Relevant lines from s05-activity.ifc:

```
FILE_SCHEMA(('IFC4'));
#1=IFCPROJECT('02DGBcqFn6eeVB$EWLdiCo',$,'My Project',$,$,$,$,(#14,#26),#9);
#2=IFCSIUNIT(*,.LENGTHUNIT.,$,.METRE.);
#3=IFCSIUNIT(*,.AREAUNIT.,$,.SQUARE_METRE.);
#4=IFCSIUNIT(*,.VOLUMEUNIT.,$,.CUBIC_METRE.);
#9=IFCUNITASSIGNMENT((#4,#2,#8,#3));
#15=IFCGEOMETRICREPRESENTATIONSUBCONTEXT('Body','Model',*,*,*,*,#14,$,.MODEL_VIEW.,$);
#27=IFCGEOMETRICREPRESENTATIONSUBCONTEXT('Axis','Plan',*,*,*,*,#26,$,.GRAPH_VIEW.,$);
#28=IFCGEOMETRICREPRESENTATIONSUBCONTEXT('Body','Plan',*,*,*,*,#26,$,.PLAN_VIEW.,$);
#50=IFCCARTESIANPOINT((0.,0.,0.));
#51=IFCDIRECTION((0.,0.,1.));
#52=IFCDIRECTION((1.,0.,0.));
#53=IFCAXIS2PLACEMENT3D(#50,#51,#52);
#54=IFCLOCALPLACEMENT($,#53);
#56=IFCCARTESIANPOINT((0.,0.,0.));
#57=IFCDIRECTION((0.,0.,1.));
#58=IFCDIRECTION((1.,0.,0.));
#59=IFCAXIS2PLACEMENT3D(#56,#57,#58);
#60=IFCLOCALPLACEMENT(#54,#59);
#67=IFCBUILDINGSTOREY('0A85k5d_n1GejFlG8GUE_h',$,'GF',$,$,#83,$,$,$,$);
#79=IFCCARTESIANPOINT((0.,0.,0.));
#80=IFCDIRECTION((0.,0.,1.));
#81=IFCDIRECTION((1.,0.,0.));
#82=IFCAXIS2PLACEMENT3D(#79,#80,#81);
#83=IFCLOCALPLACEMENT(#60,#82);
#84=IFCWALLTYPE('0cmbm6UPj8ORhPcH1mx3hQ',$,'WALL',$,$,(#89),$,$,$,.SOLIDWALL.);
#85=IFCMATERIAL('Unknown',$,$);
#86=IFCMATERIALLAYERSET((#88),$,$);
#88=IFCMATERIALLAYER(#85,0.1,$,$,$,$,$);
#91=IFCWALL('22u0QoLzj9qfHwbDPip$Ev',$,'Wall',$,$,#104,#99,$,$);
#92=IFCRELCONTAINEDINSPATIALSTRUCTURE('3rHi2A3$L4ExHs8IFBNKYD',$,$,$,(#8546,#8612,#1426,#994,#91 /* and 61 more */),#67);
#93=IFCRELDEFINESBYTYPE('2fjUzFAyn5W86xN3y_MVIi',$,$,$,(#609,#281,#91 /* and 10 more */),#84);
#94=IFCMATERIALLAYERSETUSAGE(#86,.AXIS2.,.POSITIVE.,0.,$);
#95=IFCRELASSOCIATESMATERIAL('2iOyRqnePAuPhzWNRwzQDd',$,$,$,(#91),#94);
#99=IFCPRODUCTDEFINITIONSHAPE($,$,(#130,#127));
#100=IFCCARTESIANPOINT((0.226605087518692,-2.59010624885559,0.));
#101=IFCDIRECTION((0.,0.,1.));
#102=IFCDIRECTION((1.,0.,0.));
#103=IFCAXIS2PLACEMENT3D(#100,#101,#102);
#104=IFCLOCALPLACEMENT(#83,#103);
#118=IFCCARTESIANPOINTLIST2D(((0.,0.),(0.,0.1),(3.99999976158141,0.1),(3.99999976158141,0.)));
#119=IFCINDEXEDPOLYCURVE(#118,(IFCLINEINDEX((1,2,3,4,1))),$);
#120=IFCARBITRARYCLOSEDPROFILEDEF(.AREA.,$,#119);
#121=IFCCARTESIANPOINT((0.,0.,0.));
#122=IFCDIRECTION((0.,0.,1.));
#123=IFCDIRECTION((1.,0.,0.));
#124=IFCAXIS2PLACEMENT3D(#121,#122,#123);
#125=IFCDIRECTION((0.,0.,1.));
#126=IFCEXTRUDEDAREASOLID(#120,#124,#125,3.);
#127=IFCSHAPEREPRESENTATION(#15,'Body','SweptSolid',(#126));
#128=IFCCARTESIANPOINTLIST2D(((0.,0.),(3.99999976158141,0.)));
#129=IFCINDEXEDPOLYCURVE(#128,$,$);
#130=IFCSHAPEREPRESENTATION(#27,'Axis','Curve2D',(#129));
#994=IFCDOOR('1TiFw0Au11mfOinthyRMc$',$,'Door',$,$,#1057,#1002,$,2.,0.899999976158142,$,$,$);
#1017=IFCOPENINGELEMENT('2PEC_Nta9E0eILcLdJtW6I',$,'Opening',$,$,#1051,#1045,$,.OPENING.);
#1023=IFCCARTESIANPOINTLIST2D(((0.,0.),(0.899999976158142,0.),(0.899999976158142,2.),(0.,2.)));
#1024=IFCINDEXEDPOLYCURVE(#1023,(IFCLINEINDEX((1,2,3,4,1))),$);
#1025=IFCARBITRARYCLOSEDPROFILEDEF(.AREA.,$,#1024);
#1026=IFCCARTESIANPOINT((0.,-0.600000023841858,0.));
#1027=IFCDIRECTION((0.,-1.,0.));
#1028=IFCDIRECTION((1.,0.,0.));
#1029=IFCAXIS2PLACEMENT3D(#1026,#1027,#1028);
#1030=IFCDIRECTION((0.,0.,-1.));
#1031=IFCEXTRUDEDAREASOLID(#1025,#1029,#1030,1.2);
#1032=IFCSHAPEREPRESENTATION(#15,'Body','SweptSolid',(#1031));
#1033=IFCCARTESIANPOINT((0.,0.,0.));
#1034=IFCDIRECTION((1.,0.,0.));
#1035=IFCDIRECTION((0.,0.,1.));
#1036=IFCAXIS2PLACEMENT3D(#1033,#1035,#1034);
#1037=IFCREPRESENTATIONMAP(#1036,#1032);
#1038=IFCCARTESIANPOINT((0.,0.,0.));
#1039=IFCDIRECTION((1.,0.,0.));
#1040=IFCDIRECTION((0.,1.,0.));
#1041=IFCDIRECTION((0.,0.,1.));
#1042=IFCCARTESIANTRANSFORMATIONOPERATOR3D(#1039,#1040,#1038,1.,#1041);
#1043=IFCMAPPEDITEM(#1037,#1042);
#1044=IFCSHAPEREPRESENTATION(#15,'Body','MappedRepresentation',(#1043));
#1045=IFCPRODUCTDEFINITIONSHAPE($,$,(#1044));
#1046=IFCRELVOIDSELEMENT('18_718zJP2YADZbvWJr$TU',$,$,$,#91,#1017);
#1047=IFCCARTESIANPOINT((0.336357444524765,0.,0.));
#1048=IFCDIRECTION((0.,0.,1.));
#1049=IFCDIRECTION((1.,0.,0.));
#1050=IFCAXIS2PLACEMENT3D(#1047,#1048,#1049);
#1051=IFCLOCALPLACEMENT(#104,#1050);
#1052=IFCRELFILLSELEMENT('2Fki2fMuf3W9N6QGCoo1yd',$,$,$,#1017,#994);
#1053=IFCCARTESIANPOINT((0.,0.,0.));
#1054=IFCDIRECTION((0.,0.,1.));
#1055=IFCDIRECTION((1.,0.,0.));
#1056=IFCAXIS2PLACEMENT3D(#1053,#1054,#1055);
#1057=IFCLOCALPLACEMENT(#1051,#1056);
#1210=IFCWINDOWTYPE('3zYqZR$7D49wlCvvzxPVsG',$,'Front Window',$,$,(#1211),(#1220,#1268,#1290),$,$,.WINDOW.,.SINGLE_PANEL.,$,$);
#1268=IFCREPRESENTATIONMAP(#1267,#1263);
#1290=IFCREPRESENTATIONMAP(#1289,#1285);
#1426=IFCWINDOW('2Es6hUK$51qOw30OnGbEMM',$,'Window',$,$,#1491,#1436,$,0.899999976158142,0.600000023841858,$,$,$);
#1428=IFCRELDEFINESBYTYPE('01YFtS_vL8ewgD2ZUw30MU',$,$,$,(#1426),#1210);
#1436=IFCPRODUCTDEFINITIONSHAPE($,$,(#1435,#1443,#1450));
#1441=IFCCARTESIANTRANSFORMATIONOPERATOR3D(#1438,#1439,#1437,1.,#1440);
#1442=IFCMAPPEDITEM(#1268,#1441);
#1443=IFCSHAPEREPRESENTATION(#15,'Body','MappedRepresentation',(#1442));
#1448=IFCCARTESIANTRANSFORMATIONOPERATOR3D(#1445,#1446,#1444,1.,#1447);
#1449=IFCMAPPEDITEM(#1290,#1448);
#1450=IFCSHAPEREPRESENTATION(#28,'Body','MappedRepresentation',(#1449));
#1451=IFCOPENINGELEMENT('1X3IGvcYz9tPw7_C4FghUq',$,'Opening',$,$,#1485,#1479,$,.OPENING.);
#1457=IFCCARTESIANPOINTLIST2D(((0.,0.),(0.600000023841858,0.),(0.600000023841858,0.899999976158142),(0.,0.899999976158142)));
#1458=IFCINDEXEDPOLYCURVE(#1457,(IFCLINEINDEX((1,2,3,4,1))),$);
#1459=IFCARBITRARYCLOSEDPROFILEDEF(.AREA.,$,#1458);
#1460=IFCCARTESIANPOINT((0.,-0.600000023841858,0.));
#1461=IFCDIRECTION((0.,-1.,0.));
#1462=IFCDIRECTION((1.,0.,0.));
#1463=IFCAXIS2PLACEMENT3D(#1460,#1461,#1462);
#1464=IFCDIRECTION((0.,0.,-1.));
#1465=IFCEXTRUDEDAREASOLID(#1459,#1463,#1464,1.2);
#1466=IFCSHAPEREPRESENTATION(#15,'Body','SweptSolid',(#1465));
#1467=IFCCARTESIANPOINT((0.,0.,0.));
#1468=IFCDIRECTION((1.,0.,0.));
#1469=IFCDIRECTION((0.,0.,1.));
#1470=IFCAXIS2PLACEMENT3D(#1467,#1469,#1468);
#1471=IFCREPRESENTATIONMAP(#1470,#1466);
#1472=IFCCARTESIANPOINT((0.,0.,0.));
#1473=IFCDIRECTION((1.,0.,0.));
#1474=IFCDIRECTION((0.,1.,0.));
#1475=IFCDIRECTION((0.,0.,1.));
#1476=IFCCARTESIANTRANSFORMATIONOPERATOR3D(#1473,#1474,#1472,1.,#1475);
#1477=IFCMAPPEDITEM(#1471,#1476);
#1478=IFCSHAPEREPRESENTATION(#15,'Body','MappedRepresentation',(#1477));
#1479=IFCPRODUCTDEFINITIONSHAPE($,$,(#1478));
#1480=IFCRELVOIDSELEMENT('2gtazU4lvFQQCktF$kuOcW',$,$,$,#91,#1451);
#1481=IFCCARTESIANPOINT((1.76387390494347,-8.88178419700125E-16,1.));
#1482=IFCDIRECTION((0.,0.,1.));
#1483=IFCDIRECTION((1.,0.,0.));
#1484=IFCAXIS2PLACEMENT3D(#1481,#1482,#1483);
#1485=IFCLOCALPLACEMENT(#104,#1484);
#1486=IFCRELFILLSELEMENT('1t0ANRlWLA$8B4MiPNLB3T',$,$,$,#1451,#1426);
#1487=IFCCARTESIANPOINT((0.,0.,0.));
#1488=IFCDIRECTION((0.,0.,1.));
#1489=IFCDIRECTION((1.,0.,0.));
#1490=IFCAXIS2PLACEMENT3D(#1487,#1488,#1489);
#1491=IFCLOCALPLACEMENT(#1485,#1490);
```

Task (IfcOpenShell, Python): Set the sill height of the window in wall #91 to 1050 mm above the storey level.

```python
import numpy as np
import ifcopenshell
import ifcopenshell.api.geometry
import ifcopenshell.geom
import ifcopenshell.util.element
import ifcopenshell.util.placement
import ifcopenshell.util.shape
import ifcopenshell.util.unit

model = ifcopenshell.open("s05-activity.ifc")
unit_scale = ifcopenshell.util.unit.calculate_unit_scale(model)

window = model.by_guid("2Es6hUK$51qOw30OnGbEMM")
opening = window.FillsVoids[0].RelatingOpeningElement
storey = ifcopenshell.util.element.get_container(window, ifc_class="IfcBuildingStorey")
level = ifcopenshell.util.placement.get_local_placement(storey.ObjectPlacement)[2, 3]

# The opening's origin need not be at the sill, so measure its lowest point.
shape = ifcopenshell.geom.create_shape(ifcopenshell.geom.settings(), opening)
bottom = ifcopenshell.util.shape.get_shape_bottom_elevation(shape, shape.geometry) / unit_scale
dz = level + 1.05 - bottom

shift = np.array([0.0, 0.0, dz])
# The window is placed relative to its opening, so it follows when the opening moves.
matrix = ifcopenshell.util.placement.get_local_placement(opening.ObjectPlacement)
matrix[:3, 3] += shift
ifcopenshell.api.geometry.edit_object_placement(
    model, product=opening, matrix=matrix, is_si=False, should_transform_children=True
)

print(f"moved by {dz * unit_scale:+.3f} m")

model.write("s05-activity-out.ifc")
```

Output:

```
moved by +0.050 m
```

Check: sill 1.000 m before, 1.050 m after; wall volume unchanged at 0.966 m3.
